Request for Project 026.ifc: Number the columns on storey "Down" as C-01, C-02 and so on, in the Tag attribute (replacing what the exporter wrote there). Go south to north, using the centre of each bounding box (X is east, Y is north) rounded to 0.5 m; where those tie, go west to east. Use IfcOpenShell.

First a look at what the model holds.

```python
import ifcopenshell
import ifcopenshell.util.element
import ifcopenshell.util.placement

model = ifcopenshell.open("Project 026.ifc")
print(model.schema)
storey = next(s for s in model.by_type("IfcBuildingStorey") if s.Name == "Down")
columns = [e for e in ifcopenshell.util.element.get_decomposition(storey) if e.is_a("IfcColumn")]
for e in sorted(columns, key=lambda e: e.id()):
    origin = ifcopenshell.util.placement.get_local_placement(e.ObjectPlacement)[:3, 3]
    print(e.id(), e.Tag, e.Name, origin.round(2) + 0.0, sep=" | ")
```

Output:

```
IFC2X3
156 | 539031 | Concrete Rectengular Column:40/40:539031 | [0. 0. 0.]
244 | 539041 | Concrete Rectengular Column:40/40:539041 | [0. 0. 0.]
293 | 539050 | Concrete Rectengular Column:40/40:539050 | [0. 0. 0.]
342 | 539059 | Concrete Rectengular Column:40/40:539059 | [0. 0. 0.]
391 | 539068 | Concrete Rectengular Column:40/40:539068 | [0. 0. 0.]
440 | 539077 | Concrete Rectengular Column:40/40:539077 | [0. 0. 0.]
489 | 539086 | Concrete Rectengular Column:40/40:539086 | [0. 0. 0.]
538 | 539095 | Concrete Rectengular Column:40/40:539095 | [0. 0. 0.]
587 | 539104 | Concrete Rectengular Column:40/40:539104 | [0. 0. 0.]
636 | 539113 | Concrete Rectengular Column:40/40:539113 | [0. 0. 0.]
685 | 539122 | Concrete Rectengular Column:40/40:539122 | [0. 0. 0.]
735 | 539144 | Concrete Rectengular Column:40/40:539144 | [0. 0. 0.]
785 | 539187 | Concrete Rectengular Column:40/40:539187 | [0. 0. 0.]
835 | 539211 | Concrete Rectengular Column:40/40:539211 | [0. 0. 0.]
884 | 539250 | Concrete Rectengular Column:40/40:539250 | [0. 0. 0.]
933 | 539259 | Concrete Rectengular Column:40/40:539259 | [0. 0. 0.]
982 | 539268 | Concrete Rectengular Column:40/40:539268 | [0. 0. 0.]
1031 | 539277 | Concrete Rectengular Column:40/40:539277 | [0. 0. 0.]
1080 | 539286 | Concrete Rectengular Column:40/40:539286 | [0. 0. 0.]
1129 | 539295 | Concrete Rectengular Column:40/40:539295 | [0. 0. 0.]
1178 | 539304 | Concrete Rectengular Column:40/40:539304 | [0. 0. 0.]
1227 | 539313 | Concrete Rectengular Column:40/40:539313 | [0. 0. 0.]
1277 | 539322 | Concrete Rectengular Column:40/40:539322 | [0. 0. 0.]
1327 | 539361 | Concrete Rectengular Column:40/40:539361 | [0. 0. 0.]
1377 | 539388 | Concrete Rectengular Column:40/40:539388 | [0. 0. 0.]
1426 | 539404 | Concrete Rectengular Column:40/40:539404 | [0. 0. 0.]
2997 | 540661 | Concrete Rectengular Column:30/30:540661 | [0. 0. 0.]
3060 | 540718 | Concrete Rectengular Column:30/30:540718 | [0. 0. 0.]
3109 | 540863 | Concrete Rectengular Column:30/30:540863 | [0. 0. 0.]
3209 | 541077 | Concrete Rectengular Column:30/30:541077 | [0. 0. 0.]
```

```python
import ifcopenshell
import ifcopenshell.geom
import ifcopenshell.util.element
import ifcopenshell.util.shape

model = ifcopenshell.open("Project 026.ifc")
settings = ifcopenshell.geom.settings()
settings.set("use-world-coords", True)


def centre(element):
    shape = ifcopenshell.geom.create_shape(settings, element)
    return ifcopenshell.util.shape.get_bbox_centroid(shape.geometry)


storey = next(s for s in model.by_type("IfcBuildingStorey") if s.Name == "Down")
columns = [e for e in ifcopenshell.util.element.get_decomposition(storey) if e.is_a("IfcColumn")]

# Insertion points can sit at a corner or the storey origin, so sort by the geometry (in metres).
centres = {e: centre(e) for e in columns}
columns.sort(key=lambda e: (round(centres[e][1] / 0.5), centres[e][0]))

for i, e in enumerate(columns, start=1):
    number = f"C-{i:02d}"
    e.Tag = number
    print(e.id(), number)

model.write("Project 026_edited.ifc")
```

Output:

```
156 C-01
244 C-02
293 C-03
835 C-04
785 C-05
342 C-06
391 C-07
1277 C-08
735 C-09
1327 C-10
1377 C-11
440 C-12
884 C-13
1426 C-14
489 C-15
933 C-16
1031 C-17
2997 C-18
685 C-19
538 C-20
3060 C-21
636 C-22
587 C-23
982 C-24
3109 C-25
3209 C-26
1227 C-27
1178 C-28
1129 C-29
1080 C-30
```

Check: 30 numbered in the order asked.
